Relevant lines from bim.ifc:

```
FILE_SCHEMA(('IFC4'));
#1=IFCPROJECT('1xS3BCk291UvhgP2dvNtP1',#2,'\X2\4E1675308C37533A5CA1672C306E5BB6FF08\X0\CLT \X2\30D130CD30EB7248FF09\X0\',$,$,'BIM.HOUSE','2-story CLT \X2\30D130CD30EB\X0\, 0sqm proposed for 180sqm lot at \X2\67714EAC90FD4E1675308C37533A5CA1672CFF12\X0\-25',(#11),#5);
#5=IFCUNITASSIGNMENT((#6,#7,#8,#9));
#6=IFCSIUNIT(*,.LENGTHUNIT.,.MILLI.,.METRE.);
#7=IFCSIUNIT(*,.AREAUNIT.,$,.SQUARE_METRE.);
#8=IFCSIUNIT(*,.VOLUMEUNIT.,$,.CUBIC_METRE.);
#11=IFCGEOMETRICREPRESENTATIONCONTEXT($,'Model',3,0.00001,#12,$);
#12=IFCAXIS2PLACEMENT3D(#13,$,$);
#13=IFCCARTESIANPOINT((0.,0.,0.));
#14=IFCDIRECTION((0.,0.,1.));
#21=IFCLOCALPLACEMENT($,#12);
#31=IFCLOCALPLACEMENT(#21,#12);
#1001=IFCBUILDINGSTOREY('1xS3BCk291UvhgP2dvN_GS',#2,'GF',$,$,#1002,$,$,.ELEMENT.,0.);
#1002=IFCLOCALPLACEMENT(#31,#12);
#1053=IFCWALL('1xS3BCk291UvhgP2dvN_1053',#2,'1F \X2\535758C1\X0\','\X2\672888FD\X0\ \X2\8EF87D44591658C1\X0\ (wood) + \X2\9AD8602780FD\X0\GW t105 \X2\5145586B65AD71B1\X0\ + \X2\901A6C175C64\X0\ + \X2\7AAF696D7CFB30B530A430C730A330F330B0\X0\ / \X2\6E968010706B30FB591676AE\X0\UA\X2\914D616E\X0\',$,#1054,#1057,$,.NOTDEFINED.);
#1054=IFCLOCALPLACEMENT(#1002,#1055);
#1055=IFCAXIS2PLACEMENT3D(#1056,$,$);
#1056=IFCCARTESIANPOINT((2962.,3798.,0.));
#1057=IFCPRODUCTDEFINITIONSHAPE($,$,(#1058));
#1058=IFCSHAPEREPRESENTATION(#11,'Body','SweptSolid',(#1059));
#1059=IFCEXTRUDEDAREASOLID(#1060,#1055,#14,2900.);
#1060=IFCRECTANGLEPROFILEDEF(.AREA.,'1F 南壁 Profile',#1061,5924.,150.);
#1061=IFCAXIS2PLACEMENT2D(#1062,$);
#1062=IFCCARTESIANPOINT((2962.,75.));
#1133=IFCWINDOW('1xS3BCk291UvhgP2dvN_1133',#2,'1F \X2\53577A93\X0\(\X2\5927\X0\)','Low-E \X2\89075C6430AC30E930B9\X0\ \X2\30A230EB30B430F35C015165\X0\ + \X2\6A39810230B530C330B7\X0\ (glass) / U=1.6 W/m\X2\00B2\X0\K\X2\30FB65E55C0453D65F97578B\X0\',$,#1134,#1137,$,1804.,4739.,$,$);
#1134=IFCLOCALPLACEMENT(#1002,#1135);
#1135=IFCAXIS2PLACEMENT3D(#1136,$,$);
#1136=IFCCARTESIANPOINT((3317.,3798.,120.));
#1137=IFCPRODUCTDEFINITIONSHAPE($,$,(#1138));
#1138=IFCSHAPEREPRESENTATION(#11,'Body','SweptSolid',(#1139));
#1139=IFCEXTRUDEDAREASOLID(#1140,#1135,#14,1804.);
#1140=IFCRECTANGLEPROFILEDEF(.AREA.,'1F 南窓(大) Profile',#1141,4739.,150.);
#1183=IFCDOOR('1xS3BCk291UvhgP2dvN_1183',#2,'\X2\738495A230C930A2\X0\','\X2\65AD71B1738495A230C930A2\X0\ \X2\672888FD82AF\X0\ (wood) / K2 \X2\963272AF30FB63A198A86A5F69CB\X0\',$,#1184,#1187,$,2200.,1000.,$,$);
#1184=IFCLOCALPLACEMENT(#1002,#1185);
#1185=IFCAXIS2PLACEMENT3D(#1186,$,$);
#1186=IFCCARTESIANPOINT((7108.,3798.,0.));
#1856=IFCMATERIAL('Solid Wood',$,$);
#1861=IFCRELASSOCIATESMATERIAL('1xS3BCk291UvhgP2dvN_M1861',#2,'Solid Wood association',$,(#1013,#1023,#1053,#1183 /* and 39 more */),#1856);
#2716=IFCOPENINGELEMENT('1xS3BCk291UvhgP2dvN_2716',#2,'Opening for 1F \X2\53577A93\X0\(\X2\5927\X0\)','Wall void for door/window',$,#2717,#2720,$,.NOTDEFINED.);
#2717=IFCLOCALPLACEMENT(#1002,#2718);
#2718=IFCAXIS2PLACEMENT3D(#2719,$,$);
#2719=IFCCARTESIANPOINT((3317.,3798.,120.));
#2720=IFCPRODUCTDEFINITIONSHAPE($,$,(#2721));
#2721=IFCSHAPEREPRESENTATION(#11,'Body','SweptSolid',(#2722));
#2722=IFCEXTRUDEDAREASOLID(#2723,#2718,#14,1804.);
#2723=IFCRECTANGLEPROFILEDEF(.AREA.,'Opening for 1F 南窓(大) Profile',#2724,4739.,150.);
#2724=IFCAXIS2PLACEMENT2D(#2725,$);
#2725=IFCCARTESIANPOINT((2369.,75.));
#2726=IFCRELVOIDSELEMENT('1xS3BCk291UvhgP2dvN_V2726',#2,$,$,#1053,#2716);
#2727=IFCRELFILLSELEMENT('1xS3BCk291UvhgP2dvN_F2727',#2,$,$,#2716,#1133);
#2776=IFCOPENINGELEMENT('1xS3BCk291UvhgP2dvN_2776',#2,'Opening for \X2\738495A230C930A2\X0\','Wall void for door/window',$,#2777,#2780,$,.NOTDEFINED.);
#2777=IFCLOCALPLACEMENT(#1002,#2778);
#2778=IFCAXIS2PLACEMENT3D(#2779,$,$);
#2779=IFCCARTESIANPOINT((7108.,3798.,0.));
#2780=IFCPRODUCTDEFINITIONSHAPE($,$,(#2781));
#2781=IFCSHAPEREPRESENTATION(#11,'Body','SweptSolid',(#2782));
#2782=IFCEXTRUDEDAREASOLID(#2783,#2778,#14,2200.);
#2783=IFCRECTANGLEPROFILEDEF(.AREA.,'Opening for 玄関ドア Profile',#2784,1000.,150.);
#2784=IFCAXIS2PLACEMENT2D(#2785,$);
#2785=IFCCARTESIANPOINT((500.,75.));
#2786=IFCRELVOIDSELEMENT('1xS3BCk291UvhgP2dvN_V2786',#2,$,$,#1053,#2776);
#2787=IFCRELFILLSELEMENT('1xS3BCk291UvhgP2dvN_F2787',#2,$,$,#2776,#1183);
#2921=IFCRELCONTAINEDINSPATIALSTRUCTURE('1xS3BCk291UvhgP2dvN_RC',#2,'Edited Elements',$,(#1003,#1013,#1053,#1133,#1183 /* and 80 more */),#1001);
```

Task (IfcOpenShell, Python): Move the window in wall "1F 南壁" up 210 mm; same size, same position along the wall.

```python
import numpy as np
import ifcopenshell
import ifcopenshell.api.geometry
import ifcopenshell.util.placement
import ifcopenshell.util.unit

model = ifcopenshell.open("bim.ifc")
unit_scale = ifcopenshell.util.unit.calculate_unit_scale(model)

window = model.by_guid("1xS3BCk291UvhgP2dvN_1133")
opening = window.FillsVoids[0].RelatingOpeningElement
dz = 0.21 / unit_scale

shift = np.array([0.0, 0.0, dz])
# The window is not placed relative to its opening, so move both.
for product in (opening, window):
    matrix = ifcopenshell.util.placement.get_local_placement(product.ObjectPlacement)
    matrix[:3, 3] += shift
    ifcopenshell.api.geometry.edit_object_placement(model, product=product, matrix=matrix, is_si=False)

print(f"moved by {dz * unit_scale:+.3f} m")

model.write("bim_v2.ifc")
```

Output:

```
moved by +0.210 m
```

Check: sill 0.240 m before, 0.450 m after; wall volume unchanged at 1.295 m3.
